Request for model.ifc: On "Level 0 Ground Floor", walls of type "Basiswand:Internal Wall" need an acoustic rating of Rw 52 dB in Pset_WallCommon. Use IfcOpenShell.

First a look at what the model holds.

```python
import ifcopenshell
import ifcopenshell.util.element

model = ifcopenshell.open("model.ifc")
print(model.schema)
storey = next(s for s in model.by_type("IfcBuildingStorey") if s.Name == "Level 0 Ground Floor")
walls = [e for e in ifcopenshell.util.element.get_decomposition(storey) if e.is_a("IfcWall")]
seen = {}
for e in walls:
    element_type = ifcopenshell.util.element.get_type(e)
    key = (element_type.Name if element_type != e and element_type else None, ifcopenshell.util.element.get_pset(e, "Pset_WallCommon", "AcousticRating"))
    seen[key] = seen.get(key, 0) + 1
for (name, value), count in sorted(seen.items(), key=str):
    print(count, "x", name, "|", value)
```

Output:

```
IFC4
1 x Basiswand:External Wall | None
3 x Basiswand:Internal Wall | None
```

```python
import ifcopenshell
import ifcopenshell.api.pset
import ifcopenshell.util.element

model = ifcopenshell.open("model.ifc")

storey = next(s for s in model.by_type("IfcBuildingStorey") if s.Name == "Level 0 Ground Floor")
walls = [e for e in ifcopenshell.util.element.get_decomposition(storey) if e.is_a("IfcWall")]

count = 0
for e in walls:
    element_type = ifcopenshell.util.element.get_type(e)
    if element_type in (None, e) or element_type.Name != "Basiswand:Internal Wall":
        continue
    # add_pset returns the element's existing set when there is one.
    pset = ifcopenshell.api.pset.add_pset(model, product=e, name="Pset_WallCommon")
    ifcopenshell.api.pset.edit_pset(model, pset=pset, properties={"AcousticRating": "Rw 52 dB"})
    count += 1

print(count, "walls updated")

model.write("model_updated.ifc")
```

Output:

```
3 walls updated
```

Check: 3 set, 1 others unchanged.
